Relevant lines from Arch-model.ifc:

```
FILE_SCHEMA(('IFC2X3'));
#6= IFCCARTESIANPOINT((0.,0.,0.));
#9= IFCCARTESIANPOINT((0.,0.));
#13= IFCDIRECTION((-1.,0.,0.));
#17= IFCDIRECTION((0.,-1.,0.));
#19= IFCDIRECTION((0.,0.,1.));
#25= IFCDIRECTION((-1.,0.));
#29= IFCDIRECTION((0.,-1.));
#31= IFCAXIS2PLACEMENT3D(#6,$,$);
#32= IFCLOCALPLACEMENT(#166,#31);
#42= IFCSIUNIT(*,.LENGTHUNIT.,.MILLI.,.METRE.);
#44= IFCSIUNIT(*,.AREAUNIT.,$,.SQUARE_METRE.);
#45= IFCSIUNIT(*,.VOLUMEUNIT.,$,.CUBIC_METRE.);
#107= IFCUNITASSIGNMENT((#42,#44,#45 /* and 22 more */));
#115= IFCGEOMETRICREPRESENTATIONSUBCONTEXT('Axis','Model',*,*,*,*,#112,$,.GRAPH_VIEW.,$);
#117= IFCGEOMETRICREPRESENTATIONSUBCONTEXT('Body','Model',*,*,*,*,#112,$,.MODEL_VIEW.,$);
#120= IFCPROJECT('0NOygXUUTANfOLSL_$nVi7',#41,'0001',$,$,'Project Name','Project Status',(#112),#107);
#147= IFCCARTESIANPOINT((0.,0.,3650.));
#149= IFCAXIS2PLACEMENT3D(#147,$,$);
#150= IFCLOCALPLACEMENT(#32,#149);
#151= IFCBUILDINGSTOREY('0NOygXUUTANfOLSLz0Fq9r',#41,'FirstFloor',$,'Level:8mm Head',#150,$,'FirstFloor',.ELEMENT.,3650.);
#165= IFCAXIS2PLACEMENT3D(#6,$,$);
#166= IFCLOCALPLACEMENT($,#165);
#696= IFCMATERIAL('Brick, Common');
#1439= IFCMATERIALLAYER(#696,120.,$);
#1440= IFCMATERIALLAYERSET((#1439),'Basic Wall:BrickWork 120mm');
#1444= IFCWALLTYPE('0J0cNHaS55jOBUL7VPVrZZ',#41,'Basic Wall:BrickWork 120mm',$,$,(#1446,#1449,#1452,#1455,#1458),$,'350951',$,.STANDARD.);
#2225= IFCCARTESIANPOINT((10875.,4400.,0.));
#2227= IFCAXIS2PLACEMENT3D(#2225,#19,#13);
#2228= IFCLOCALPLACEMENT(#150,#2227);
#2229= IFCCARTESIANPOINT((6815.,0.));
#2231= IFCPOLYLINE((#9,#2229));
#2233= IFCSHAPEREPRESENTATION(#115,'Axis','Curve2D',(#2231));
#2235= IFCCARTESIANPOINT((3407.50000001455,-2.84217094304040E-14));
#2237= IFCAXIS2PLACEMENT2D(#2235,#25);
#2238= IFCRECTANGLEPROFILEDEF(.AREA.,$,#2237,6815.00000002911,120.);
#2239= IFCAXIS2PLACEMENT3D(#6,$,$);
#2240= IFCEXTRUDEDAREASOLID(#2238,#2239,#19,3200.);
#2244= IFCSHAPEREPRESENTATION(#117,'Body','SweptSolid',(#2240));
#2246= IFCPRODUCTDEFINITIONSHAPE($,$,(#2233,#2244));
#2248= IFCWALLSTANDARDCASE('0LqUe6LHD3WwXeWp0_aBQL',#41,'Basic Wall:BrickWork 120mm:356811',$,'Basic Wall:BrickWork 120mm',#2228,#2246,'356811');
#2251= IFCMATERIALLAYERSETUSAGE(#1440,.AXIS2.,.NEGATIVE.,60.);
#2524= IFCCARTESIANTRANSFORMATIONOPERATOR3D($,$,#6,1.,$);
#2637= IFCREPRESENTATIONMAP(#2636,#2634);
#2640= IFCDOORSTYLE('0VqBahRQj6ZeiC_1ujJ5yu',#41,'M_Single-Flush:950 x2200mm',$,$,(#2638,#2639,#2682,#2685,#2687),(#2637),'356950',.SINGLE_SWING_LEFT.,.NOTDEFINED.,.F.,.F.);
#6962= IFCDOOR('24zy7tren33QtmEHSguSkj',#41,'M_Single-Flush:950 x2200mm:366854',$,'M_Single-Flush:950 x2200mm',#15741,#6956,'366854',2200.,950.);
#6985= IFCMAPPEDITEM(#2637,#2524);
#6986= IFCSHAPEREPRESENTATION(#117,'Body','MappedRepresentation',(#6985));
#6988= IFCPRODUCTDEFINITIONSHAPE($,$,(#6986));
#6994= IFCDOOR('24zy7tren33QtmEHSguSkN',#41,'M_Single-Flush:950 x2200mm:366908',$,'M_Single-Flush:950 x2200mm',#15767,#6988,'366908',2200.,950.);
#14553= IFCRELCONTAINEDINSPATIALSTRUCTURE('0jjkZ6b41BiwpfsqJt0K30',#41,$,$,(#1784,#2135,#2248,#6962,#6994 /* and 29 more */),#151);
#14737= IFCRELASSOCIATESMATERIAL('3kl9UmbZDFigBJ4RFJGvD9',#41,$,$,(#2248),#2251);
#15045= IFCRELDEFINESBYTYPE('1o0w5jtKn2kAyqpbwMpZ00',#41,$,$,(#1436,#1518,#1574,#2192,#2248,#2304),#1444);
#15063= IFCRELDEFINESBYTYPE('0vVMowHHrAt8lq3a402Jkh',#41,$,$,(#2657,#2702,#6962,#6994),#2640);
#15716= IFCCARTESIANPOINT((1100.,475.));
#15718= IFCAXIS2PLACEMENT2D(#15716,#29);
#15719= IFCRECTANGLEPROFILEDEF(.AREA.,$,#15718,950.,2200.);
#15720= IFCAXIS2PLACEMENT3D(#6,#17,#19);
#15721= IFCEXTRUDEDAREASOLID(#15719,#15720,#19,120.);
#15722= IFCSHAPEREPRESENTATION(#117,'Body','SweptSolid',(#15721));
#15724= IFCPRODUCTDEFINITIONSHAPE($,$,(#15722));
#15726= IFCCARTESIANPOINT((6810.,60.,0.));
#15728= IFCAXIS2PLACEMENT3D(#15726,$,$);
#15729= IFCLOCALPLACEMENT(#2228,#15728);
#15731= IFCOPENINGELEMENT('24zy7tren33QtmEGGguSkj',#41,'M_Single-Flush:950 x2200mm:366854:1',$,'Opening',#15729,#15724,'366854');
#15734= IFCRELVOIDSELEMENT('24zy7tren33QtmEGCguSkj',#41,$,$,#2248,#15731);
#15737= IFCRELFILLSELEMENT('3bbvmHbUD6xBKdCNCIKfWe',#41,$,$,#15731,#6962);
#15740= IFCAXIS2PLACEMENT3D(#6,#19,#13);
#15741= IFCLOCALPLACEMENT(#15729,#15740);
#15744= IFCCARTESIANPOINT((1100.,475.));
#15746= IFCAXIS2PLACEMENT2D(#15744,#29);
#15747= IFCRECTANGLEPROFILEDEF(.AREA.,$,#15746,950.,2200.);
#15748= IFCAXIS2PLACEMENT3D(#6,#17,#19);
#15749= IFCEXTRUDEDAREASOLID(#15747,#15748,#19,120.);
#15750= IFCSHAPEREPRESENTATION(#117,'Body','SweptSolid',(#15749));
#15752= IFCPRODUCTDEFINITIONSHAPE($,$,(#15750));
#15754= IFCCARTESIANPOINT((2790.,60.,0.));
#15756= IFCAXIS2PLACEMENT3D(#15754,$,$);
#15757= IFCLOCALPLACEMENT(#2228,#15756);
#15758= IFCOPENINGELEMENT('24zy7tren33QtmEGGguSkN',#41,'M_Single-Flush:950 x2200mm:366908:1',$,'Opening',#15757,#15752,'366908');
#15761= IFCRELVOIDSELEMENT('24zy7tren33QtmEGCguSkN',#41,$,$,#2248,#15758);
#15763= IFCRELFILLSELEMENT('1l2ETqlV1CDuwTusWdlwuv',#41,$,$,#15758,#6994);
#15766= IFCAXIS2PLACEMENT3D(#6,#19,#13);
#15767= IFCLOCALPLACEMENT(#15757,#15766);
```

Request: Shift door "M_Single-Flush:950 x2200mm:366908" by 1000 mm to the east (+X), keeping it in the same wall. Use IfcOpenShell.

```python
import ifcopenshell
import ifcopenshell.api.geometry
import ifcopenshell.util.placement
import ifcopenshell.util.unit

model = ifcopenshell.open("Arch-model.ifc")
unit_scale = ifcopenshell.util.unit.calculate_unit_scale(model)

door = model.by_guid("24zy7tren33QtmEHSguSkN")
opening = door.FillsVoids[0].RelatingOpeningElement
wall = opening.VoidsElements[0].RelatingBuildingElement

wall_matrix = ifcopenshell.util.placement.get_local_placement(wall.ObjectPlacement)
shift = wall_matrix[:3, 0] * -1 / unit_scale
before = ifcopenshell.util.placement.get_local_placement(door.ObjectPlacement)[:3, 3].copy()

# The door is placed relative to its opening, so it follows when the opening moves.
matrix = ifcopenshell.util.placement.get_local_placement(opening.ObjectPlacement)
matrix[:3, 3] += shift
ifcopenshell.api.geometry.edit_object_placement(
    model, product=opening, matrix=matrix, is_si=False, should_transform_children=True
)

after = ifcopenshell.util.placement.get_local_placement(door.ObjectPlacement)[:3, 3]
print("door moved by", (after - before).round(3) + 0.0)

model.write("Arch-model-out.ifc")
```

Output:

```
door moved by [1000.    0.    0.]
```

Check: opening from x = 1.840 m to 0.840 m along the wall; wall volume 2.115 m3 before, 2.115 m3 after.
